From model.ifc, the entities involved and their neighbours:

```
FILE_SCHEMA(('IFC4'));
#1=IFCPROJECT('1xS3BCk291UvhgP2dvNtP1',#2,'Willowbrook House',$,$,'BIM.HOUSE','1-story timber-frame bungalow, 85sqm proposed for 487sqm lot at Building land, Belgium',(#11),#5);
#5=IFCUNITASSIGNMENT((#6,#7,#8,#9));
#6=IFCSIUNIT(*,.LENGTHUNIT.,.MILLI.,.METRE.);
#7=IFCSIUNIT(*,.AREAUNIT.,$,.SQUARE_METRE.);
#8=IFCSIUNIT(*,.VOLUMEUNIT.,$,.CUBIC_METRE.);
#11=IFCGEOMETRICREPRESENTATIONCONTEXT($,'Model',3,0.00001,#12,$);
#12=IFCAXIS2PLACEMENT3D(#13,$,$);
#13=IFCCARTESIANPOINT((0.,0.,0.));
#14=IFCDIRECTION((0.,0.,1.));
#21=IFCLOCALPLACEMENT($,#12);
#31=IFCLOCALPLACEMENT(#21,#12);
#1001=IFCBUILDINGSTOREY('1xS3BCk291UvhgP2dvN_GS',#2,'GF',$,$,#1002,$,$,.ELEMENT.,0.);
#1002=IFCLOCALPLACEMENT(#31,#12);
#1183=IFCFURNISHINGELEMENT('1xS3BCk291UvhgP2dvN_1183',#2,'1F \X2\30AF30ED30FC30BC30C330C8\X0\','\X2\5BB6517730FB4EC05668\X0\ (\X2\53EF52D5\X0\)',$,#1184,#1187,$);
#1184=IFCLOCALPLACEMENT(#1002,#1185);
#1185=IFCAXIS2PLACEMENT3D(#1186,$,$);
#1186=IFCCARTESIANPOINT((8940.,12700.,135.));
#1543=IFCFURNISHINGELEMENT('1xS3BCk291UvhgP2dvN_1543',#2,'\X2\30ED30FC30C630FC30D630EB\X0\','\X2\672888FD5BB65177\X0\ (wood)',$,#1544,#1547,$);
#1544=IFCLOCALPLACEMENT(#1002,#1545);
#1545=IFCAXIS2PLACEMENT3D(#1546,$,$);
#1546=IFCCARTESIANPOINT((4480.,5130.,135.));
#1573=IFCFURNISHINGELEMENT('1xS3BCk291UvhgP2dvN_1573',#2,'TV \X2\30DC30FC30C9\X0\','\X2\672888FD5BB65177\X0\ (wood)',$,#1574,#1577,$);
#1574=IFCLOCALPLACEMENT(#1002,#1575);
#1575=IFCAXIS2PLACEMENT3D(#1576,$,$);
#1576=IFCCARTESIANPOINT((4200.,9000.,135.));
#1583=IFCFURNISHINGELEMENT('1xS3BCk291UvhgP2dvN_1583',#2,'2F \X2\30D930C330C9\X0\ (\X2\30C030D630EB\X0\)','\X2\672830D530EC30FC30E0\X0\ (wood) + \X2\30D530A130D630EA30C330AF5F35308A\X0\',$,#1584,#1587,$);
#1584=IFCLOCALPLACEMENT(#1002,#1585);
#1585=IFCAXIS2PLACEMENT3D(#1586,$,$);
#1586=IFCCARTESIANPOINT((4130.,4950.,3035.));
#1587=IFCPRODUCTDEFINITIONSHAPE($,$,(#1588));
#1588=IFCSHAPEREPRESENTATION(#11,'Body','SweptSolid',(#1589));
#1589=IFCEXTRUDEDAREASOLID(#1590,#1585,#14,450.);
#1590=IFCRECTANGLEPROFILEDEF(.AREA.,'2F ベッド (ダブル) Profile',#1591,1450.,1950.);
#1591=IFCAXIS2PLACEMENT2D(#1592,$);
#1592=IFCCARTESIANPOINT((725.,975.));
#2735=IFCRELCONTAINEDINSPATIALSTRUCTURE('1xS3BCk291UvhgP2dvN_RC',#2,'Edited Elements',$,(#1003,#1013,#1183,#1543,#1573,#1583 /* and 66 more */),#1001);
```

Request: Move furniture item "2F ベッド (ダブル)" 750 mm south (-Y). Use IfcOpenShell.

```python
import ifcopenshell
import ifcopenshell.api.geometry
import ifcopenshell.util.placement
import ifcopenshell.util.unit

model = ifcopenshell.open("model.ifc")
unit_scale = ifcopenshell.util.unit.calculate_unit_scale(model)

item = model.by_guid("1xS3BCk291UvhgP2dvN_1583")
matrix = ifcopenshell.util.placement.get_local_placement(item.ObjectPlacement)
matrix[1, 3] -= 0.75 / unit_scale
ifcopenshell.api.geometry.edit_object_placement(model, product=item, matrix=matrix, is_si=False)

print(ifcopenshell.util.placement.get_local_placement(item.ObjectPlacement).round(3) + 0.0)

model.write("model_rev.ifc")
```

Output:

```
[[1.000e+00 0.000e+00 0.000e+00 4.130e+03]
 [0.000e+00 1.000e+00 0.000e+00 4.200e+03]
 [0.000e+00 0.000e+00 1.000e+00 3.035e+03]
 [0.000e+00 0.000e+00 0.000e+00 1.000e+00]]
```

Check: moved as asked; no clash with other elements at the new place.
